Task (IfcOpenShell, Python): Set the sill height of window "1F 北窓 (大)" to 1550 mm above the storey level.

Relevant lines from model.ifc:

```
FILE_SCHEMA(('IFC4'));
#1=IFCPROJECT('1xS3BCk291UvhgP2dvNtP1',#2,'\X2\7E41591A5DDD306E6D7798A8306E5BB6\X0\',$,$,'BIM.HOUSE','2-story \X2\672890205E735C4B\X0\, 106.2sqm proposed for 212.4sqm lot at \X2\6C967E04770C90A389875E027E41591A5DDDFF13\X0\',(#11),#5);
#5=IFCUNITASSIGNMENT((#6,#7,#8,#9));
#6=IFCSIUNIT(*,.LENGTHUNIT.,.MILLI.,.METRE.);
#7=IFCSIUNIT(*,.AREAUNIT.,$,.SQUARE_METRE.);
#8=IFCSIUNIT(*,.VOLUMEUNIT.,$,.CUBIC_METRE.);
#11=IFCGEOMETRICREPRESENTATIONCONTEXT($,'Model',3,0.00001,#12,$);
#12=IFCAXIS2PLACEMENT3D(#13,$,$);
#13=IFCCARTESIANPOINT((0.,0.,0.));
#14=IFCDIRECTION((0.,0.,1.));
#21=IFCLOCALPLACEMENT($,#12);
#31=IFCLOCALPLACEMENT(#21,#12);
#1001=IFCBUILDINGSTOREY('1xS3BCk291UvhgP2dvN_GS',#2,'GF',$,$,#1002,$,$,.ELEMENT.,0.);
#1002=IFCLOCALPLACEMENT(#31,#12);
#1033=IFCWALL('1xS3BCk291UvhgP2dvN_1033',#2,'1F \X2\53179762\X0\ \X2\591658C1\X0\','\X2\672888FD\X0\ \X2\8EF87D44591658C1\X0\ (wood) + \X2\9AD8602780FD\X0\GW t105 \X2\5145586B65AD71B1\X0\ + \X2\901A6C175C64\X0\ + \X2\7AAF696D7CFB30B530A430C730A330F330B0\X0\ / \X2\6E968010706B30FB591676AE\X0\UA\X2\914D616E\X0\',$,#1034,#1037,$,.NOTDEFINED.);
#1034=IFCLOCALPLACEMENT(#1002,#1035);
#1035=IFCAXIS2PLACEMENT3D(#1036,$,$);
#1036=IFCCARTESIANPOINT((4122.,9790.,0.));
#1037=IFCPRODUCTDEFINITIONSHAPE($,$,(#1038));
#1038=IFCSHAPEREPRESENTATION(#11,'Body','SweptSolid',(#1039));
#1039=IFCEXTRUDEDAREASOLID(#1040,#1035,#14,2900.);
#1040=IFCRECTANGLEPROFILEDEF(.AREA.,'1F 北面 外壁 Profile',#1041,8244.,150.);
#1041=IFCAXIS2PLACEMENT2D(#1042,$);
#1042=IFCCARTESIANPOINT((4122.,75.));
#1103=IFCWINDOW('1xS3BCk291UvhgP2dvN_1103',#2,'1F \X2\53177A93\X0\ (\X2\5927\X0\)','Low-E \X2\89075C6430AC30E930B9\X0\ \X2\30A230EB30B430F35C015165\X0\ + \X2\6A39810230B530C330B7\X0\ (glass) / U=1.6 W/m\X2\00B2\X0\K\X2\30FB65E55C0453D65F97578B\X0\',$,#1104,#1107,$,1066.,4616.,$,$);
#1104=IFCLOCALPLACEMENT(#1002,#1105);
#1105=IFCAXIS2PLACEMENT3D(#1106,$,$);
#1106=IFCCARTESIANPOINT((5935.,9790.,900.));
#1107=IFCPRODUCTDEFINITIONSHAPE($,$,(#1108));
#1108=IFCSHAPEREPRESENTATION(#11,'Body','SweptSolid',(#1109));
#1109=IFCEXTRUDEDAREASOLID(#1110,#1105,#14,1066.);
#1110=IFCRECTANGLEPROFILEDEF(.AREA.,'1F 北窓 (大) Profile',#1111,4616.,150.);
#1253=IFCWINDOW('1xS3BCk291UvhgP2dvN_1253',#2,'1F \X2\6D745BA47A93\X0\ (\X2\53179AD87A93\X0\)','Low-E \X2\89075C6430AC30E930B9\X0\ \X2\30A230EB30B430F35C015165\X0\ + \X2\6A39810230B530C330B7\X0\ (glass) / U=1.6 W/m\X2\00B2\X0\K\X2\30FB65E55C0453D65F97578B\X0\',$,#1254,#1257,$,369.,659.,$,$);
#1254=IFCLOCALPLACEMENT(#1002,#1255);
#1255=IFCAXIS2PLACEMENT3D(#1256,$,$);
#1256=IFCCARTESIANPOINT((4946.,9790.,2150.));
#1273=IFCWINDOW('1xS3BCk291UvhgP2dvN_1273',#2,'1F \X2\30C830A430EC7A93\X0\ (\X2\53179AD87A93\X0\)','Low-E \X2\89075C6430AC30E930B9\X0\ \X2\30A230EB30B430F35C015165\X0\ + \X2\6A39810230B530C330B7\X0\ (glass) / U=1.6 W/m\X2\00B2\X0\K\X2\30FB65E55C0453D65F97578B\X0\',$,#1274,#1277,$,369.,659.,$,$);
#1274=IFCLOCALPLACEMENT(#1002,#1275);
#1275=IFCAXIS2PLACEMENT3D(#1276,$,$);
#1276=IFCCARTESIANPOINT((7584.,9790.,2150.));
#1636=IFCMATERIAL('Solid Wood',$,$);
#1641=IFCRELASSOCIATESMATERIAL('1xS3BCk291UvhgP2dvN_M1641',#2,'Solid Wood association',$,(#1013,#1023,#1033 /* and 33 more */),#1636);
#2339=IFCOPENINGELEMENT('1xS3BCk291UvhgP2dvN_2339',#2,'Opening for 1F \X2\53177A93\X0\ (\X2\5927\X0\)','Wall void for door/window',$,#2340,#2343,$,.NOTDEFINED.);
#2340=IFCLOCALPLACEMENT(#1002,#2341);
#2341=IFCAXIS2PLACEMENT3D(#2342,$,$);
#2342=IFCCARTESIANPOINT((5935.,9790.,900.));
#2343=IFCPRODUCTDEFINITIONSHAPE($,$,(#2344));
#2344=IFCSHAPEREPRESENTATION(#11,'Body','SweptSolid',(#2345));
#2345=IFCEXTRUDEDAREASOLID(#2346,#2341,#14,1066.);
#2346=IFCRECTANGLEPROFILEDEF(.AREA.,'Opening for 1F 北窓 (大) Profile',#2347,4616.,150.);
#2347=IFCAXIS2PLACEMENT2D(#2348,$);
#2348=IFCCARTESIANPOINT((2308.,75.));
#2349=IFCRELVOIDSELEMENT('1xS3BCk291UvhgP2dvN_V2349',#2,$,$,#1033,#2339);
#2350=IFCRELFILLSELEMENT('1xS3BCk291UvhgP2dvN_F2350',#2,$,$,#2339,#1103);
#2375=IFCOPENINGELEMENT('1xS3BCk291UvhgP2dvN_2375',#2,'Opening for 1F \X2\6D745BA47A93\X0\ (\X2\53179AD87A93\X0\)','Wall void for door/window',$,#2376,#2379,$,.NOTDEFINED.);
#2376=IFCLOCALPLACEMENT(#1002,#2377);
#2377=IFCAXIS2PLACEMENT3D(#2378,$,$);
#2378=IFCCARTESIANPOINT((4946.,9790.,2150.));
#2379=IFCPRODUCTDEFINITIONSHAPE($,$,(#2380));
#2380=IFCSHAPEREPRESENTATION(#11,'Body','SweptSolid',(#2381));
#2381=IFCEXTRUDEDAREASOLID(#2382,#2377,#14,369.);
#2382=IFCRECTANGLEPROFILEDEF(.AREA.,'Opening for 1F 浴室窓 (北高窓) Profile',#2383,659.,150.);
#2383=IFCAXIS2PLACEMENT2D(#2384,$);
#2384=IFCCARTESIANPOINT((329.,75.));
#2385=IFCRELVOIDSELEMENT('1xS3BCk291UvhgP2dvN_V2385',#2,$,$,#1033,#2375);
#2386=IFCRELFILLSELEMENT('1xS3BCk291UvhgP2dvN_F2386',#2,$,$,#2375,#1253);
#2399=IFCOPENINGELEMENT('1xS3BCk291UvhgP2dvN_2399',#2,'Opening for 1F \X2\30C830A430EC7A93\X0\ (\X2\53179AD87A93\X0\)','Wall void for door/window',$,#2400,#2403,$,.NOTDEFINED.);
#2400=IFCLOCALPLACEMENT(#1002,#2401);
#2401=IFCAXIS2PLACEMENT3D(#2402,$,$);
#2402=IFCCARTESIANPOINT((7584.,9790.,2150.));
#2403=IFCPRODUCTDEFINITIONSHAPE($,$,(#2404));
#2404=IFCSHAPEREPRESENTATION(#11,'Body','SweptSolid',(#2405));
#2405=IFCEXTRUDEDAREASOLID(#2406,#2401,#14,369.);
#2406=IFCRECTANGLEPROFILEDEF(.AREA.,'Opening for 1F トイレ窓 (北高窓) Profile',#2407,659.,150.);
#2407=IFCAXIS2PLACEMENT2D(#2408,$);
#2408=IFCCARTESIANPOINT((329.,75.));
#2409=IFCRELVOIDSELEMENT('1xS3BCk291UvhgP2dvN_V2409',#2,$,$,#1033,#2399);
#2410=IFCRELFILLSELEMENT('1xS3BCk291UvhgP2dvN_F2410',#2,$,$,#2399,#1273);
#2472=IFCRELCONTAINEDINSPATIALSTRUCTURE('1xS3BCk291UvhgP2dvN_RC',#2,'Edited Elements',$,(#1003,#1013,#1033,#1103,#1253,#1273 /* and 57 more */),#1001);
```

```python
import numpy as np
import ifcopenshell
import ifcopenshell.api.geometry
import ifcopenshell.geom
import ifcopenshell.util.element
import ifcopenshell.util.placement
import ifcopenshell.util.shape
import ifcopenshell.util.unit

model = ifcopenshell.open("model.ifc")
unit_scale = ifcopenshell.util.unit.calculate_unit_scale(model)

window = model.by_guid("1xS3BCk291UvhgP2dvN_1103")
opening = window.FillsVoids[0].RelatingOpeningElement
storey = ifcopenshell.util.element.get_container(window, ifc_class="IfcBuildingStorey")
level = ifcopenshell.util.placement.get_local_placement(storey.ObjectPlacement)[2, 3]

# The opening's origin need not be at the sill, so measure its lowest point.
shape = ifcopenshell.geom.create_shape(ifcopenshell.geom.settings(), opening)
bottom = ifcopenshell.util.shape.get_shape_bottom_elevation(shape, shape.geometry) / unit_scale
dz = level + 1.55 / unit_scale - bottom

shift = np.array([0.0, 0.0, dz])
# The window is not placed relative to its opening, so move both.
for product in (opening, window):
    matrix = ifcopenshell.util.placement.get_local_placement(product.ObjectPlacement)
    matrix[:3, 3] += shift
    ifcopenshell.api.geometry.edit_object_placement(model, product=product, matrix=matrix, is_si=False)

print(f"moved by {dz * unit_scale:+.3f} m")

model.write("model_rev.ifc")
```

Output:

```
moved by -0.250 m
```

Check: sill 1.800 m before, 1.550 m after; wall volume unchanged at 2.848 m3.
